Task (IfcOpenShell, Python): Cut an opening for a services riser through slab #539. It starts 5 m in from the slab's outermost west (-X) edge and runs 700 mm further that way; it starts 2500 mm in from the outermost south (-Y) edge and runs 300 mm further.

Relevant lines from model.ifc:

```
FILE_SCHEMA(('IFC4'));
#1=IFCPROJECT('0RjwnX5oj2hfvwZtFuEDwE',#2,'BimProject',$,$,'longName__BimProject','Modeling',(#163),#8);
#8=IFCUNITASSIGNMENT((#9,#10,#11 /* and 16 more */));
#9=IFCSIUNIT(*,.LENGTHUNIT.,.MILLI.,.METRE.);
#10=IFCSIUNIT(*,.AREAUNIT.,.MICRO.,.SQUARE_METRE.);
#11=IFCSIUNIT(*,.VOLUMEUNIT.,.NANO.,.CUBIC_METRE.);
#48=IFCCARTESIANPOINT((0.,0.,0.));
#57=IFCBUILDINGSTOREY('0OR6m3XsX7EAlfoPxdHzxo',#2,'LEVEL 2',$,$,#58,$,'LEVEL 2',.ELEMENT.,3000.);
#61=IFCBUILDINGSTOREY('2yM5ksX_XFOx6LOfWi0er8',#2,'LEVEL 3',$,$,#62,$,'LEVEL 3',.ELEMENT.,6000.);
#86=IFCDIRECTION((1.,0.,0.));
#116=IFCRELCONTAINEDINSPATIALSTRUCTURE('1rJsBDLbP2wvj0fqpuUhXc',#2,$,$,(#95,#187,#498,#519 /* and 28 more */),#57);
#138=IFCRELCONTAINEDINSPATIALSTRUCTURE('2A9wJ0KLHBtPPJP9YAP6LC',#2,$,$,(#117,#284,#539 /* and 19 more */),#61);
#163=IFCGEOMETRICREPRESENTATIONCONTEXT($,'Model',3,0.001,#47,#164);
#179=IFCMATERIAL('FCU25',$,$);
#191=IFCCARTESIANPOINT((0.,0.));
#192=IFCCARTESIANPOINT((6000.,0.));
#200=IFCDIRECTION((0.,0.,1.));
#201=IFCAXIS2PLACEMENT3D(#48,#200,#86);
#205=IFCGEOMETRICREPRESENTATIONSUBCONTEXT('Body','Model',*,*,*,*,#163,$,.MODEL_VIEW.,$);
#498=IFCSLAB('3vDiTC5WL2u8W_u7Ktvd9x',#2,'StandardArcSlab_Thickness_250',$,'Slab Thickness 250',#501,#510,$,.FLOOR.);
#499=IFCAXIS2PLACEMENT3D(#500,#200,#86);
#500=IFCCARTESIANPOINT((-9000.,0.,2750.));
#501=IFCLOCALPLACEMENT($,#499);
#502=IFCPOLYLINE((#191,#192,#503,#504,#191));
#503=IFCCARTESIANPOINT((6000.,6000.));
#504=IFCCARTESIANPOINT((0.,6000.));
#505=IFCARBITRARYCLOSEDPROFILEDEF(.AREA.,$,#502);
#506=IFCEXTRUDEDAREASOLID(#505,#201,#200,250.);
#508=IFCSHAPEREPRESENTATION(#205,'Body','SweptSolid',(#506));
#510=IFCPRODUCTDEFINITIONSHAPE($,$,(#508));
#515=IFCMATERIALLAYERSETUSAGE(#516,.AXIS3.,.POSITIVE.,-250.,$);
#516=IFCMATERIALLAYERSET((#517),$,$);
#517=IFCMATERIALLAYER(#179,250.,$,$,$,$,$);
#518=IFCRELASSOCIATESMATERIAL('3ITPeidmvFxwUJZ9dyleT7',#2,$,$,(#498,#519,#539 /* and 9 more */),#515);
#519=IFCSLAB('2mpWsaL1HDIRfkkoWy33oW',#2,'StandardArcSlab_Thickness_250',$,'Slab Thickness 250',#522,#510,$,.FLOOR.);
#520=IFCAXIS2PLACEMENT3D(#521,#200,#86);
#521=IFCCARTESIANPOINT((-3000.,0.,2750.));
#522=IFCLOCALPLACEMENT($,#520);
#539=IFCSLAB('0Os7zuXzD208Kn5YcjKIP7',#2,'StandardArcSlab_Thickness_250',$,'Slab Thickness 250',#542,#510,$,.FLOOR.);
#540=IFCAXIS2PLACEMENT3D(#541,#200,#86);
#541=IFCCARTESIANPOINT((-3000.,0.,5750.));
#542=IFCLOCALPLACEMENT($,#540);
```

```python
import numpy as np
import ifcopenshell
import ifcopenshell.api.feature
import ifcopenshell.api.geometry
import ifcopenshell.api.root
import ifcopenshell.geom
import ifcopenshell.util.placement
import ifcopenshell.util.representation
import ifcopenshell.util.shape
import ifcopenshell.util.unit

model = ifcopenshell.open("model.ifc")
unit_scale = ifcopenshell.util.unit.calculate_unit_scale(model)
settings = ifcopenshell.geom.settings()


def volume(element):
    """Net volume in cubic metres, openings subtracted."""
    shape = ifcopenshell.geom.create_shape(settings, element)
    return ifcopenshell.util.shape.get_volume(shape.geometry)


slab = model.by_guid("0Os7zuXzD208Kn5YcjKIP7")
before = volume(slab)

# Extent in the slab's own axes, in metres. The edges named are its -X and -Y sides.
slab_shape = ifcopenshell.geom.create_shape(settings, slab)
vertices = ifcopenshell.util.shape.get_vertices(slab_shape.geometry)
x_min, y_min, bottom = vertices.min(axis=0)
top = vertices[:, 2].max()

opening = ifcopenshell.api.root.create_entity(model, ifc_class="IfcOpeningElement", name="Services riser opening", predefined_type="OPENING")
context = ifcopenshell.util.representation.get_context(model, "Model", "Body", "MODEL_VIEW")
width, depth = 0.7, 0.3
outline = [(0.0, 0.0), (width, 0.0), (width, depth), (0.0, depth), (0.0, 0.0)]
# Overshoot both faces by 50 mm so the cut is clean.
shape = ifcopenshell.api.geometry.add_slab_representation(
    model, context=context, depth=top - bottom + 0.1, polyline=outline
)
ifcopenshell.api.geometry.assign_representation(model, product=opening, representation=shape)

matrix = ifcopenshell.util.placement.get_local_placement(slab.ObjectPlacement)
matrix[:, 3] = matrix @ np.append(np.array([x_min + 5, y_min + 2.5, bottom - 0.05]) / unit_scale, 1.0)
ifcopenshell.api.geometry.edit_object_placement(model, product=opening, matrix=matrix, is_si=False)
ifcopenshell.api.feature.add_feature(model, feature=opening, element=slab)

after = volume(slab)

print(f"slab volume {before:.3f} -> {after:.3f} m3")

model.write("model_updated.ifc")
```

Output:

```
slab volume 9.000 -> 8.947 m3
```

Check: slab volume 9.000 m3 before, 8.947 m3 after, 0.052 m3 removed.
